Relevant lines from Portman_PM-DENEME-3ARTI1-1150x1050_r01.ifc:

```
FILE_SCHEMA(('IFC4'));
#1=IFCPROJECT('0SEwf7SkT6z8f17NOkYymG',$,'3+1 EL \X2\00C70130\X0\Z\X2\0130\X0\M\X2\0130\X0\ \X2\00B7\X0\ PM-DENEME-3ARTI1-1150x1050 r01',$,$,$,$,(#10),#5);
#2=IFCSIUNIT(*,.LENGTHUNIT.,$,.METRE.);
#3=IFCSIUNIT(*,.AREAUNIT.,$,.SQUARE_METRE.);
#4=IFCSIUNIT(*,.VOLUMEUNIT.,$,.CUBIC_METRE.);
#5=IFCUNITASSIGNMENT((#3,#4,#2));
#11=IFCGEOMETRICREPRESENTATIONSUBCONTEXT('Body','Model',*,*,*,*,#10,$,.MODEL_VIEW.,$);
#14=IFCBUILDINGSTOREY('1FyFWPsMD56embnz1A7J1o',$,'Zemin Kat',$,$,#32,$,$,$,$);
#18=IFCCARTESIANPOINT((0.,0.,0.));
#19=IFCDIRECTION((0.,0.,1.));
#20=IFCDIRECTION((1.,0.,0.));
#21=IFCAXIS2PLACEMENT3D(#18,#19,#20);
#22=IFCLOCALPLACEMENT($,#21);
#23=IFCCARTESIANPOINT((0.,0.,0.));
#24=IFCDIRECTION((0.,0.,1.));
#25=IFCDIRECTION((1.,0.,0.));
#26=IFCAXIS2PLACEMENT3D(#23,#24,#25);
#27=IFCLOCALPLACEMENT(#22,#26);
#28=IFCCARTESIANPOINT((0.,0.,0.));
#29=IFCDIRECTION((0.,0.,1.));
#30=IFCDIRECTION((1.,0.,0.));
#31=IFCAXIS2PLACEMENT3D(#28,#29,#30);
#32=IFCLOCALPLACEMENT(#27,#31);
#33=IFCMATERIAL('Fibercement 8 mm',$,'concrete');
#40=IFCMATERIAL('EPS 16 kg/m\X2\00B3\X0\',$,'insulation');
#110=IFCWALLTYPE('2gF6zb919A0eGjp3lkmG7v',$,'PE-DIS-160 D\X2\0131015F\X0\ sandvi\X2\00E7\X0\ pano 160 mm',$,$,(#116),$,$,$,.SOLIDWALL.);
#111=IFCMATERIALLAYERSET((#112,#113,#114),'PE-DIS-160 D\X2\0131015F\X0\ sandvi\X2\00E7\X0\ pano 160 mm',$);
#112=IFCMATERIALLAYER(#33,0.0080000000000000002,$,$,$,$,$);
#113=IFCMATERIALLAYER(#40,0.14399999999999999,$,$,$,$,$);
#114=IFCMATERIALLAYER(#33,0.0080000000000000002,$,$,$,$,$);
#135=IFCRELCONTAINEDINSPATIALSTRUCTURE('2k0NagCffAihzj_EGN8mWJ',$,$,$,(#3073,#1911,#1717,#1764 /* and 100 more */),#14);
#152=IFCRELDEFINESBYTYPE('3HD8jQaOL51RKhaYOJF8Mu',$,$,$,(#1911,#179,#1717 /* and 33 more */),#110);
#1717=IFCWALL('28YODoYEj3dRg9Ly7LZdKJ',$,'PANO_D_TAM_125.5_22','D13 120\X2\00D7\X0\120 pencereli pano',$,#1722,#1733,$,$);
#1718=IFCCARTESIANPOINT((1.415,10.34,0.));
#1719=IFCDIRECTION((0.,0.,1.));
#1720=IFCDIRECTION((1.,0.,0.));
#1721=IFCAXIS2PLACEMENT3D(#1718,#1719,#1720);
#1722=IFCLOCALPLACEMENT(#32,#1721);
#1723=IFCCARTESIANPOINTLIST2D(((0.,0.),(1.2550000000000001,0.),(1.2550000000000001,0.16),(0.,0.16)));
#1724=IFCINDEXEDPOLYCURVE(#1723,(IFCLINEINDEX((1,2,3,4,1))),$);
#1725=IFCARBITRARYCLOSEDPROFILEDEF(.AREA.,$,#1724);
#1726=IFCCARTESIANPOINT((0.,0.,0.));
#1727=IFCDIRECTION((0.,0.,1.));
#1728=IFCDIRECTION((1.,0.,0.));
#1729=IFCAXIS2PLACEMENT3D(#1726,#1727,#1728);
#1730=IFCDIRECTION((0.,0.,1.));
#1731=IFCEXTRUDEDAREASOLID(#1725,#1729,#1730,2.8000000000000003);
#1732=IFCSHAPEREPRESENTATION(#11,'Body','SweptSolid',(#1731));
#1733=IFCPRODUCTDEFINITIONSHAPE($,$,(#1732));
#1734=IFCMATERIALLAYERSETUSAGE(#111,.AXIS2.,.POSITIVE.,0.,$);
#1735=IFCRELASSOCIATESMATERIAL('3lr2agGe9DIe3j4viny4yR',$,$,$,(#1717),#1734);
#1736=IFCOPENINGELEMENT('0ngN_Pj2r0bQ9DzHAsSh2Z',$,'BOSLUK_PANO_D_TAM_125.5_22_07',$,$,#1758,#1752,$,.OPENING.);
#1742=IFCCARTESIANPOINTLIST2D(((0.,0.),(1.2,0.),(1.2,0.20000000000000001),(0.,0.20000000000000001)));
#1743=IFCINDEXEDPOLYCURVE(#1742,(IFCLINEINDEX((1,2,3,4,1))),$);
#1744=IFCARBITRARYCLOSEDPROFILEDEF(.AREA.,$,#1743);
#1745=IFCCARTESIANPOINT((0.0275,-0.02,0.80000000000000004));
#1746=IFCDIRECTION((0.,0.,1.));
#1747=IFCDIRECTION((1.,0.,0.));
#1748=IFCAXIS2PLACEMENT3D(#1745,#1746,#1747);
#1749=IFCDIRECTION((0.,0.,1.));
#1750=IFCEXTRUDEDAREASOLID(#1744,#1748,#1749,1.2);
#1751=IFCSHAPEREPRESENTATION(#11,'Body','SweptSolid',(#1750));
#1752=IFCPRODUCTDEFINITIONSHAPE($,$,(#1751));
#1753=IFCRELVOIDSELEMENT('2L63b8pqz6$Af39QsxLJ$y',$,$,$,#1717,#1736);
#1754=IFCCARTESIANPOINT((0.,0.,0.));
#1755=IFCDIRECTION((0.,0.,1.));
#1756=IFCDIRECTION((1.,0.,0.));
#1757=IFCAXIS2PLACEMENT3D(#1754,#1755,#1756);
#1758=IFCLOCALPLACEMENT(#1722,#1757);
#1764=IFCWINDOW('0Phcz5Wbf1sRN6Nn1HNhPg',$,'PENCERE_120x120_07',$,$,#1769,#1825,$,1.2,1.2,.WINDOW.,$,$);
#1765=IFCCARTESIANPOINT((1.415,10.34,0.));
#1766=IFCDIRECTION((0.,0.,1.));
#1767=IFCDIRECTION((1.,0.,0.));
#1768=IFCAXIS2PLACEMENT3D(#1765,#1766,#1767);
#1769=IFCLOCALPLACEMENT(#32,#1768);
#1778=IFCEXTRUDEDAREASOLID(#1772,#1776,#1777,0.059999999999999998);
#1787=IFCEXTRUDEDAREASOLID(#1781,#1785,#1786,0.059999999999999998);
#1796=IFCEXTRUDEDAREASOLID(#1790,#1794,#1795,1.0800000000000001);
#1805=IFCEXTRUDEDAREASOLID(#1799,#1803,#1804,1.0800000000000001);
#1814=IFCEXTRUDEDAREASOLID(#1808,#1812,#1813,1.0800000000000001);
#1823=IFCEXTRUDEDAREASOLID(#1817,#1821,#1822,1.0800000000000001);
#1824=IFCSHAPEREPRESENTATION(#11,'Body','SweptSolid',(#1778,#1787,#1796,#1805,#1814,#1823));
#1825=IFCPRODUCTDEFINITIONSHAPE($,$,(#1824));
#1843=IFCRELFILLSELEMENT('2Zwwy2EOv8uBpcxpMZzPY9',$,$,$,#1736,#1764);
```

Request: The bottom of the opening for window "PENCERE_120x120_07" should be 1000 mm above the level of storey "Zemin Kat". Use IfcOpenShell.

```python
import numpy as np
import ifcopenshell
import ifcopenshell.api.geometry
import ifcopenshell.geom
import ifcopenshell.util.element
import ifcopenshell.util.placement
import ifcopenshell.util.shape
import ifcopenshell.util.unit

model = ifcopenshell.open("Portman_PM-DENEME-3ARTI1-1150x1050_r01.ifc")
unit_scale = ifcopenshell.util.unit.calculate_unit_scale(model)

window = model.by_id(1764)
opening = window.FillsVoids[0].RelatingOpeningElement
storey = ifcopenshell.util.element.get_container(window, ifc_class="IfcBuildingStorey")
level = ifcopenshell.util.placement.get_local_placement(storey.ObjectPlacement)[2, 3]

# The opening's origin need not be at the sill, so measure its lowest point.
shape = ifcopenshell.geom.create_shape(ifcopenshell.geom.settings(), opening)
bottom = ifcopenshell.util.shape.get_shape_bottom_elevation(shape, shape.geometry) / unit_scale
dz = level + 1 / unit_scale - bottom

shift = np.array([0.0, 0.0, dz])
# The window is not placed relative to its opening, so move both.
for product in (opening, window):
    matrix = ifcopenshell.util.placement.get_local_placement(product.ObjectPlacement)
    matrix[:3, 3] += shift
    ifcopenshell.api.geometry.edit_object_placement(model, product=product, matrix=matrix, is_si=False)

print(f"moved by {dz * unit_scale:+.3f} m")

model.write("Portman_PM-DENEME-3ARTI1-1150x1050_r01_updated.ifc")
```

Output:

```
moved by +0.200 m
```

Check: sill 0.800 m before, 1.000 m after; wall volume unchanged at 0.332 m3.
